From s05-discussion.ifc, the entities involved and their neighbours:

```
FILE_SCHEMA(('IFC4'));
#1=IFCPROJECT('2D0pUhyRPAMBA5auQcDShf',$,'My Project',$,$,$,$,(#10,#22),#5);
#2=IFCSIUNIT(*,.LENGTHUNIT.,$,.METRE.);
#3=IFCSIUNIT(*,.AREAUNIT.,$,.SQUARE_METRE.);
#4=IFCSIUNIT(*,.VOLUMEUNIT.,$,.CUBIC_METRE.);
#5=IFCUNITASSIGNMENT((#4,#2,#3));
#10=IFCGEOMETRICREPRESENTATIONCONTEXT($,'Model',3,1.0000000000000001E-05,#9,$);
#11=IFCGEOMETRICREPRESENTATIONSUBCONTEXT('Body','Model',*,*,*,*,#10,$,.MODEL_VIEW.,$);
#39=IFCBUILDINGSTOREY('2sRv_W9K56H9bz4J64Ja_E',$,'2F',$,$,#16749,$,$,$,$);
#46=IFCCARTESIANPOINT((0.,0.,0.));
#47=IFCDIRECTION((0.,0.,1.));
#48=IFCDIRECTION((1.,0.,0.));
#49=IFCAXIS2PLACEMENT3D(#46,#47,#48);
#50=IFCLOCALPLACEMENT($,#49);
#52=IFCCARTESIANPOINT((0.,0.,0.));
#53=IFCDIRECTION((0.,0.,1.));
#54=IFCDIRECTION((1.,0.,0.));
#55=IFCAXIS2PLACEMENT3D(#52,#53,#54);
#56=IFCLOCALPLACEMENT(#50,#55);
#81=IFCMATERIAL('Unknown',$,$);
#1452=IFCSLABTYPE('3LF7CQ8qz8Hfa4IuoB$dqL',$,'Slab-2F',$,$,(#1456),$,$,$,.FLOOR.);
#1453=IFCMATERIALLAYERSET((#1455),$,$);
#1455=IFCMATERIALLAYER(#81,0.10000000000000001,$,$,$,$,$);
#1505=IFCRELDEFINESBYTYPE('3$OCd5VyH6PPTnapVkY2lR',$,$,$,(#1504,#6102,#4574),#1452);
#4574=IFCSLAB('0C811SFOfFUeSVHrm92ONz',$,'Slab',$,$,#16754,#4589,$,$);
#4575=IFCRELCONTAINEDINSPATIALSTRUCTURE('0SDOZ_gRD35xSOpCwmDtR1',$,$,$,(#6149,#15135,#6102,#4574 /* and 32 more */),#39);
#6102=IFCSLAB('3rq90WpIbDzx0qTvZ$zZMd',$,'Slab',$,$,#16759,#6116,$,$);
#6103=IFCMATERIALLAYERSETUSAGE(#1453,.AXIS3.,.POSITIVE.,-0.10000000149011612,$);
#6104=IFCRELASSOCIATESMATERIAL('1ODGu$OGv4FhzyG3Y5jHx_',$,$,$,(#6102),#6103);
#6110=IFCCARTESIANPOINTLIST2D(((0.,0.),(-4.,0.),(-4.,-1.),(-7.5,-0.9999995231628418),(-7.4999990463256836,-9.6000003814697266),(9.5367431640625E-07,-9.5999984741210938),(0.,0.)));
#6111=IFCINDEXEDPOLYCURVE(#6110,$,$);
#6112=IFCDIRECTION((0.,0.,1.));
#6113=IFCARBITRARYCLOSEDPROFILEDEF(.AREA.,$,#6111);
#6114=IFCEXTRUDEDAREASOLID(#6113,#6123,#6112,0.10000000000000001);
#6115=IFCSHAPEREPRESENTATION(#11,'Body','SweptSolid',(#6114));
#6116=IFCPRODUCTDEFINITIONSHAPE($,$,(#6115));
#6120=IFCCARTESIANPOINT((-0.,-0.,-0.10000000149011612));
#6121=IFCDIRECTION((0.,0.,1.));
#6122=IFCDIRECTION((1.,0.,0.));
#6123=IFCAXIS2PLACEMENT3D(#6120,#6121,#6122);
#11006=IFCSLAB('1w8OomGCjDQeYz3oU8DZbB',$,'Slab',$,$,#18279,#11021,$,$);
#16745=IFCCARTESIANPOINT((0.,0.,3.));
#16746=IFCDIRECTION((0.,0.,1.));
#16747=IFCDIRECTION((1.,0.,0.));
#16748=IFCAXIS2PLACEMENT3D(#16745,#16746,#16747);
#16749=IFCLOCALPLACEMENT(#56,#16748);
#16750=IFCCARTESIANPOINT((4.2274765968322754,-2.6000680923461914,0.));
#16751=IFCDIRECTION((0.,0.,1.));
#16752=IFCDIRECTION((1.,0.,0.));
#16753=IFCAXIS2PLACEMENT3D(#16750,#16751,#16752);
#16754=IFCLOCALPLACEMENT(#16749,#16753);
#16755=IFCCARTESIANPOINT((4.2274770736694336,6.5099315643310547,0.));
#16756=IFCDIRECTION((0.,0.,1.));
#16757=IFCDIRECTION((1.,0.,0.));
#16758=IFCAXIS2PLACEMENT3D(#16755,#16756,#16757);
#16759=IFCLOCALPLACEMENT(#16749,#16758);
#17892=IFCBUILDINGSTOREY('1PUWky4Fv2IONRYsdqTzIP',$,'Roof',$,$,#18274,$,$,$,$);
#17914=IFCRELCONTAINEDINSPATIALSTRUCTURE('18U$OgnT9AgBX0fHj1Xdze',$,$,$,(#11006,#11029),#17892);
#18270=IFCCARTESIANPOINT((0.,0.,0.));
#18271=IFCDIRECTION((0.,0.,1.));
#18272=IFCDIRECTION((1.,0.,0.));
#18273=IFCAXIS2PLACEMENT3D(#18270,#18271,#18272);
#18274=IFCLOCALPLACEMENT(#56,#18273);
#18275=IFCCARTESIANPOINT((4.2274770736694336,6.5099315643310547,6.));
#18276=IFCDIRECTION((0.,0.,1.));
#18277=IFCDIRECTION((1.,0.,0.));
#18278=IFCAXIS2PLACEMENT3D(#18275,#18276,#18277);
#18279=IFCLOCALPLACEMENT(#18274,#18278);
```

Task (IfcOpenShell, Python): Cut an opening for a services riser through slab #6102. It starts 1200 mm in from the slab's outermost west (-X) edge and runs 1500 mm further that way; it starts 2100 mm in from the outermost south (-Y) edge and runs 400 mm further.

```python
import numpy as np
import ifcopenshell
import ifcopenshell.api.feature
import ifcopenshell.api.geometry
import ifcopenshell.api.root
import ifcopenshell.geom
import ifcopenshell.util.placement
import ifcopenshell.util.representation
import ifcopenshell.util.shape
import ifcopenshell.util.unit

model = ifcopenshell.open("s05-discussion.ifc")
unit_scale = ifcopenshell.util.unit.calculate_unit_scale(model)
settings = ifcopenshell.geom.settings()


def volume(element):
    """Net volume in cubic metres, openings subtracted."""
    shape = ifcopenshell.geom.create_shape(settings, element)
    return ifcopenshell.util.shape.get_volume(shape.geometry)


slab = model.by_guid("3rq90WpIbDzx0qTvZ$zZMd")
before = volume(slab)

# Extent in the slab's own axes, in metres. The edges named are its -X and -Y sides.
slab_shape = ifcopenshell.geom.create_shape(settings, slab)
vertices = ifcopenshell.util.shape.get_vertices(slab_shape.geometry)
x_min, y_min, bottom = vertices.min(axis=0)
top = vertices[:, 2].max()

opening = ifcopenshell.api.root.create_entity(model, ifc_class="IfcOpeningElement", name="Services riser opening", predefined_type="OPENING")
context = ifcopenshell.util.representation.get_context(model, "Model", "Body", "MODEL_VIEW")
width, depth = 1.5, 0.4
outline = [(0.0, 0.0), (width, 0.0), (width, depth), (0.0, depth), (0.0, 0.0)]
# Overshoot both faces by 50 mm so the cut is clean.
shape = ifcopenshell.api.geometry.add_slab_representation(
    model, context=context, depth=top - bottom + 0.1, polyline=outline
)
ifcopenshell.api.geometry.assign_representation(model, product=opening, representation=shape)

matrix = ifcopenshell.util.placement.get_local_placement(slab.ObjectPlacement)
matrix[:, 3] = matrix @ np.append(np.array([x_min + 1.2, y_min + 2.1, bottom - 0.05]) / unit_scale, 1.0)
ifcopenshell.api.geometry.edit_object_placement(model, product=opening, matrix=matrix, is_si=False)
ifcopenshell.api.feature.add_feature(model, feature=opening, element=slab)

after = volume(slab)

print(f"slab volume {before:.3f} -> {after:.3f} m3")

model.write("s05-discussion-out.ifc")
```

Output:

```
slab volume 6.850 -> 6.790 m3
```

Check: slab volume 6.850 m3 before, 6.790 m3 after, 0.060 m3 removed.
